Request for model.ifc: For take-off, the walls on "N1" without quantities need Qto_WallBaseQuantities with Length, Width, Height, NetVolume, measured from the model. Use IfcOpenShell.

First a look at what the model holds.

```python
import ifcopenshell
import ifcopenshell.util.element
import ifcopenshell.util.unit

model = ifcopenshell.open("model.ifc")
print(model.schema)
for unit_type in ("LENGTHUNIT", "AREAUNIT", "VOLUMEUNIT"):
    print(unit_type, ifcopenshell.util.unit.calculate_unit_scale(model, unit_type))
storey = next(s for s in model.by_type("IfcBuildingStorey") if s.Name == "N1")
walls = [e for e in ifcopenshell.util.element.get_decomposition(storey) if e.is_a("IfcWall")]
for e in sorted(walls, key=lambda e: e.id()):
    print(e.id(), e.is_a(), e.Name, list(ifcopenshell.util.element.get_psets(e, qtos_only=True)), sep=" | ")
```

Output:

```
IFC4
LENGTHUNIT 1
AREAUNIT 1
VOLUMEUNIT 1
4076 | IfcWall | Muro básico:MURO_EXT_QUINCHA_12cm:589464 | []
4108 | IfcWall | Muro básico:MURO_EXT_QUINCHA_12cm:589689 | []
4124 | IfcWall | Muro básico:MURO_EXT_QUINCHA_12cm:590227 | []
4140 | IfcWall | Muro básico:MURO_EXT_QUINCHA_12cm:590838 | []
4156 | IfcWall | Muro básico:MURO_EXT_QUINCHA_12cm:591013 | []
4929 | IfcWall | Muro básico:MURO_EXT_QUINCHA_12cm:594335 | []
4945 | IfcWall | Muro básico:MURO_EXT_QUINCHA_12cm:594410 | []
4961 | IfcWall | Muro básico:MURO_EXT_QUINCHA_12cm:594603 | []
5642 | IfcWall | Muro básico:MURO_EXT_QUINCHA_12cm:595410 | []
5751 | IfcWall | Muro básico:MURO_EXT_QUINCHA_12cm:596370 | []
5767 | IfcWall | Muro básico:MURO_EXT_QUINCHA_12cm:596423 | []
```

```python
import ifcopenshell
import ifcopenshell.api.pset
import ifcopenshell.geom
import ifcopenshell.util.element
import ifcopenshell.util.shape
import ifcopenshell.util.unit

model = ifcopenshell.open("model.ifc")
unit_scale = ifcopenshell.util.unit.calculate_unit_scale(model)
volume_scale = ifcopenshell.util.unit.calculate_unit_scale(model, "VOLUMEUNIT")
settings = ifcopenshell.geom.settings()

storey = next(s for s in model.by_type("IfcBuildingStorey") if s.Name == "N1")
walls = [e for e in ifcopenshell.util.element.get_decomposition(storey) if e.is_a("IfcWall")]

for e in sorted(walls, key=lambda e: e.id()):
    if ifcopenshell.util.element.get_psets(e, qtos_only=True, should_inherit=False):
        continue
    # Geometry comes back in metres, in the element's own axes.
    shape = ifcopenshell.geom.create_shape(settings, e)
    values = {
        "Length": ifcopenshell.util.shape.get_x(shape.geometry) / unit_scale,
        "Width": ifcopenshell.util.shape.get_y(shape.geometry) / unit_scale,
        "Height": ifcopenshell.util.shape.get_z(shape.geometry) / unit_scale,
        "NetVolume": ifcopenshell.util.shape.get_volume(shape.geometry) / volume_scale,
    }
    qto = ifcopenshell.api.pset.add_qto(model, product=e, name="Qto_WallBaseQuantities")
    ifcopenshell.api.pset.edit_qto(model, qto=qto, properties=values)
    print(e.id(), {k: round(v, 3) for k, v in values.items()})

model.write("model_updated.ifc")
```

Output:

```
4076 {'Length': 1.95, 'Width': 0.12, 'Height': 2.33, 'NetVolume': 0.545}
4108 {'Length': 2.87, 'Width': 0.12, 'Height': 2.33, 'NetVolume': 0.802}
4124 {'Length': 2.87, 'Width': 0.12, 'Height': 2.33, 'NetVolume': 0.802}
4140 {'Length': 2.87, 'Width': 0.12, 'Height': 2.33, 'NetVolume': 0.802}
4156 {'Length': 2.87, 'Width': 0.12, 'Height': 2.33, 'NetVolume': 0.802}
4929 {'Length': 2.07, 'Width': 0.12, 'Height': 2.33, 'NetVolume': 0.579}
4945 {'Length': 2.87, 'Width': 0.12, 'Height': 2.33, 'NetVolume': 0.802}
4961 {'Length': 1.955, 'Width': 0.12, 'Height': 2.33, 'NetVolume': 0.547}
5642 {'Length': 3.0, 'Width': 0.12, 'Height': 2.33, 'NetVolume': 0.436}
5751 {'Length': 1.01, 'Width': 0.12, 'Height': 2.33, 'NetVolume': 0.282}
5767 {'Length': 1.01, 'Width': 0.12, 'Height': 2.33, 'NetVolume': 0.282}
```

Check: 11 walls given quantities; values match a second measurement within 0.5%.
